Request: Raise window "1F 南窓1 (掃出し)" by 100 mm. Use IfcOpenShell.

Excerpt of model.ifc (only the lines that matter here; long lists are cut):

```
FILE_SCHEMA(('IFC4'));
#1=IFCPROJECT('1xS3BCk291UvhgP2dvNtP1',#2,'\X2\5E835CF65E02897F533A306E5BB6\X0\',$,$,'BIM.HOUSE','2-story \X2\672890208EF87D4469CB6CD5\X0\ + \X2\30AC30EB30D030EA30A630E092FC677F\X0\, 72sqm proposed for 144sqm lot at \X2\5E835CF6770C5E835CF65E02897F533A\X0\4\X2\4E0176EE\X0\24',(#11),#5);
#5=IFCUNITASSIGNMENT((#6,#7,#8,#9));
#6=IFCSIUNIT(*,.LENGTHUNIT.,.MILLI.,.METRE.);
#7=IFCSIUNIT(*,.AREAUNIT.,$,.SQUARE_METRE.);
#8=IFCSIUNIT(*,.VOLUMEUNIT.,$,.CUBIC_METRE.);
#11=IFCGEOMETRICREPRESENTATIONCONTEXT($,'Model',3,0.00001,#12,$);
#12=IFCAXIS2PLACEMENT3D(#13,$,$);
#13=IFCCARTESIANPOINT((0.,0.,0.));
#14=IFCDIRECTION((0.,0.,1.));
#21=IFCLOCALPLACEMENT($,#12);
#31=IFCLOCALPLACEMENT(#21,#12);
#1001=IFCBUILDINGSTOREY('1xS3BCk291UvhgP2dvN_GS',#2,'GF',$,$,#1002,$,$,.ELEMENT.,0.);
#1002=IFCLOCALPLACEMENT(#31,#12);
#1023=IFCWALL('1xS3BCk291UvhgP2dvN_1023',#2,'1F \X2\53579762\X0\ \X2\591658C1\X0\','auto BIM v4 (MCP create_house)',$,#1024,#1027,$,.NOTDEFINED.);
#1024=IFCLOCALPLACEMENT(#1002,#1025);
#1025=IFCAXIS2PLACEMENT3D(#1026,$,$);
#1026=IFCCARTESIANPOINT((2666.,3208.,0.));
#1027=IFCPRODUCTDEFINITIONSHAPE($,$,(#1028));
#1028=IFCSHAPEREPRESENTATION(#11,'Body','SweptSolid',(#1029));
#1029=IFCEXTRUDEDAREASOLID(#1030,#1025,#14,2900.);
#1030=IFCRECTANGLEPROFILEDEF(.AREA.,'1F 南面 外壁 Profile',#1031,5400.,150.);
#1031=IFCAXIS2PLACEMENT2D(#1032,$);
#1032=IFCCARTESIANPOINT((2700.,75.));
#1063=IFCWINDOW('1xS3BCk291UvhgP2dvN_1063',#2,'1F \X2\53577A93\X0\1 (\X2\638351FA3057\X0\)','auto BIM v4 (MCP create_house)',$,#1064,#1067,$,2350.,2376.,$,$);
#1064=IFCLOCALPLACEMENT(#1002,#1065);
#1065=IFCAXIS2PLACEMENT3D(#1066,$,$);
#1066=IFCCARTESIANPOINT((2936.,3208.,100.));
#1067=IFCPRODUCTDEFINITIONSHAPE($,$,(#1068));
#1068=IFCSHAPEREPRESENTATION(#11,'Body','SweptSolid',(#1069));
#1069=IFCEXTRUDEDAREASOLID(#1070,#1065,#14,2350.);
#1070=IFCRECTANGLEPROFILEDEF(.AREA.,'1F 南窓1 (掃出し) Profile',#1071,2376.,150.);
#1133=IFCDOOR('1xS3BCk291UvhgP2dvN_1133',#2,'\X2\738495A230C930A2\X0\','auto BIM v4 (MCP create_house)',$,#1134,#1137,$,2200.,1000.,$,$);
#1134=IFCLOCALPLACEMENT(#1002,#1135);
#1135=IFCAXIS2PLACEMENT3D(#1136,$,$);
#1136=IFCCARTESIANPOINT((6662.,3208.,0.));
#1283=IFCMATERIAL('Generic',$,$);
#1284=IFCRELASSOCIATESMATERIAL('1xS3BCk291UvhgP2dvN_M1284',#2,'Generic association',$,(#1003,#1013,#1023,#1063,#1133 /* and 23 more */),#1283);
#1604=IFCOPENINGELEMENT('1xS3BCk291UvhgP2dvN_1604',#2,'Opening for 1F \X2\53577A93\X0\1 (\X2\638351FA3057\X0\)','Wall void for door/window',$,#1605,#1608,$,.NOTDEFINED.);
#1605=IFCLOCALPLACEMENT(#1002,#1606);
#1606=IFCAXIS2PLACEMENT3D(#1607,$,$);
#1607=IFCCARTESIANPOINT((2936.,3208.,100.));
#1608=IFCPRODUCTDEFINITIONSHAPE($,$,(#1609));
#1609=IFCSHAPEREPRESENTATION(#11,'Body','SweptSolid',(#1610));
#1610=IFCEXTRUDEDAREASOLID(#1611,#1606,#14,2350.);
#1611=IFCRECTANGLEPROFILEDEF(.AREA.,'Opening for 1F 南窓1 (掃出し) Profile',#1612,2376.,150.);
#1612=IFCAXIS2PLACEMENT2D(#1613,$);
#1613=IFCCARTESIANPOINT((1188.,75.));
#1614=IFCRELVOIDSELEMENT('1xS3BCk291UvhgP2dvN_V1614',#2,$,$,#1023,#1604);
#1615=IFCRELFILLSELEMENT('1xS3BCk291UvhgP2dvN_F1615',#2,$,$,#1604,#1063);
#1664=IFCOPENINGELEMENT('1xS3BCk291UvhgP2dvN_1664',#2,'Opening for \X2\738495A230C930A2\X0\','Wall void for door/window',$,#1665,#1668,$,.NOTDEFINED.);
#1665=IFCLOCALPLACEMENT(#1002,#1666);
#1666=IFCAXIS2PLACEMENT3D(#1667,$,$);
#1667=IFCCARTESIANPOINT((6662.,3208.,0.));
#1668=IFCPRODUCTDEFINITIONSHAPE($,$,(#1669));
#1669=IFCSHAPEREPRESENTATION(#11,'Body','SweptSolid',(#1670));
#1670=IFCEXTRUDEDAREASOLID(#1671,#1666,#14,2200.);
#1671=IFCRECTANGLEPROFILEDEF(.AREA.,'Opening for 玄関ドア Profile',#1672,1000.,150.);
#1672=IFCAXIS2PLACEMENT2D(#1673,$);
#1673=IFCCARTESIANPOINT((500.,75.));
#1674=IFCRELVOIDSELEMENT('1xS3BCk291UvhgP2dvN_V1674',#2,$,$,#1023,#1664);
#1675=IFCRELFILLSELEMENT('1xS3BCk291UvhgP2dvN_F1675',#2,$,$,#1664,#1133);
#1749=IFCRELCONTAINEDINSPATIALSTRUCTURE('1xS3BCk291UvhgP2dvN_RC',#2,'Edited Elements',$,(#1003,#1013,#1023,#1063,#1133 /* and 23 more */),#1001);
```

```python
import numpy as np
import ifcopenshell
import ifcopenshell.api.geometry
import ifcopenshell.util.placement
import ifcopenshell.util.unit

model = ifcopenshell.open("model.ifc")
unit_scale = ifcopenshell.util.unit.calculate_unit_scale(model)

window = model.by_id(1063)
opening = window.FillsVoids[0].RelatingOpeningElement
dz = 0.1 / unit_scale

shift = np.array([0.0, 0.0, dz])
# The window is not placed relative to its opening, so move both.
for product in (opening, window):
    matrix = ifcopenshell.util.placement.get_local_placement(product.ObjectPlacement)
    matrix[:3, 3] += shift
    ifcopenshell.api.geometry.edit_object_placement(model, product=product, matrix=matrix, is_si=False)

print(f"moved by {dz * unit_scale:+.3f} m")

model.write("model_v2.ifc")
```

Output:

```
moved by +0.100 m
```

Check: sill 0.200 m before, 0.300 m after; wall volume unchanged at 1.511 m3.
